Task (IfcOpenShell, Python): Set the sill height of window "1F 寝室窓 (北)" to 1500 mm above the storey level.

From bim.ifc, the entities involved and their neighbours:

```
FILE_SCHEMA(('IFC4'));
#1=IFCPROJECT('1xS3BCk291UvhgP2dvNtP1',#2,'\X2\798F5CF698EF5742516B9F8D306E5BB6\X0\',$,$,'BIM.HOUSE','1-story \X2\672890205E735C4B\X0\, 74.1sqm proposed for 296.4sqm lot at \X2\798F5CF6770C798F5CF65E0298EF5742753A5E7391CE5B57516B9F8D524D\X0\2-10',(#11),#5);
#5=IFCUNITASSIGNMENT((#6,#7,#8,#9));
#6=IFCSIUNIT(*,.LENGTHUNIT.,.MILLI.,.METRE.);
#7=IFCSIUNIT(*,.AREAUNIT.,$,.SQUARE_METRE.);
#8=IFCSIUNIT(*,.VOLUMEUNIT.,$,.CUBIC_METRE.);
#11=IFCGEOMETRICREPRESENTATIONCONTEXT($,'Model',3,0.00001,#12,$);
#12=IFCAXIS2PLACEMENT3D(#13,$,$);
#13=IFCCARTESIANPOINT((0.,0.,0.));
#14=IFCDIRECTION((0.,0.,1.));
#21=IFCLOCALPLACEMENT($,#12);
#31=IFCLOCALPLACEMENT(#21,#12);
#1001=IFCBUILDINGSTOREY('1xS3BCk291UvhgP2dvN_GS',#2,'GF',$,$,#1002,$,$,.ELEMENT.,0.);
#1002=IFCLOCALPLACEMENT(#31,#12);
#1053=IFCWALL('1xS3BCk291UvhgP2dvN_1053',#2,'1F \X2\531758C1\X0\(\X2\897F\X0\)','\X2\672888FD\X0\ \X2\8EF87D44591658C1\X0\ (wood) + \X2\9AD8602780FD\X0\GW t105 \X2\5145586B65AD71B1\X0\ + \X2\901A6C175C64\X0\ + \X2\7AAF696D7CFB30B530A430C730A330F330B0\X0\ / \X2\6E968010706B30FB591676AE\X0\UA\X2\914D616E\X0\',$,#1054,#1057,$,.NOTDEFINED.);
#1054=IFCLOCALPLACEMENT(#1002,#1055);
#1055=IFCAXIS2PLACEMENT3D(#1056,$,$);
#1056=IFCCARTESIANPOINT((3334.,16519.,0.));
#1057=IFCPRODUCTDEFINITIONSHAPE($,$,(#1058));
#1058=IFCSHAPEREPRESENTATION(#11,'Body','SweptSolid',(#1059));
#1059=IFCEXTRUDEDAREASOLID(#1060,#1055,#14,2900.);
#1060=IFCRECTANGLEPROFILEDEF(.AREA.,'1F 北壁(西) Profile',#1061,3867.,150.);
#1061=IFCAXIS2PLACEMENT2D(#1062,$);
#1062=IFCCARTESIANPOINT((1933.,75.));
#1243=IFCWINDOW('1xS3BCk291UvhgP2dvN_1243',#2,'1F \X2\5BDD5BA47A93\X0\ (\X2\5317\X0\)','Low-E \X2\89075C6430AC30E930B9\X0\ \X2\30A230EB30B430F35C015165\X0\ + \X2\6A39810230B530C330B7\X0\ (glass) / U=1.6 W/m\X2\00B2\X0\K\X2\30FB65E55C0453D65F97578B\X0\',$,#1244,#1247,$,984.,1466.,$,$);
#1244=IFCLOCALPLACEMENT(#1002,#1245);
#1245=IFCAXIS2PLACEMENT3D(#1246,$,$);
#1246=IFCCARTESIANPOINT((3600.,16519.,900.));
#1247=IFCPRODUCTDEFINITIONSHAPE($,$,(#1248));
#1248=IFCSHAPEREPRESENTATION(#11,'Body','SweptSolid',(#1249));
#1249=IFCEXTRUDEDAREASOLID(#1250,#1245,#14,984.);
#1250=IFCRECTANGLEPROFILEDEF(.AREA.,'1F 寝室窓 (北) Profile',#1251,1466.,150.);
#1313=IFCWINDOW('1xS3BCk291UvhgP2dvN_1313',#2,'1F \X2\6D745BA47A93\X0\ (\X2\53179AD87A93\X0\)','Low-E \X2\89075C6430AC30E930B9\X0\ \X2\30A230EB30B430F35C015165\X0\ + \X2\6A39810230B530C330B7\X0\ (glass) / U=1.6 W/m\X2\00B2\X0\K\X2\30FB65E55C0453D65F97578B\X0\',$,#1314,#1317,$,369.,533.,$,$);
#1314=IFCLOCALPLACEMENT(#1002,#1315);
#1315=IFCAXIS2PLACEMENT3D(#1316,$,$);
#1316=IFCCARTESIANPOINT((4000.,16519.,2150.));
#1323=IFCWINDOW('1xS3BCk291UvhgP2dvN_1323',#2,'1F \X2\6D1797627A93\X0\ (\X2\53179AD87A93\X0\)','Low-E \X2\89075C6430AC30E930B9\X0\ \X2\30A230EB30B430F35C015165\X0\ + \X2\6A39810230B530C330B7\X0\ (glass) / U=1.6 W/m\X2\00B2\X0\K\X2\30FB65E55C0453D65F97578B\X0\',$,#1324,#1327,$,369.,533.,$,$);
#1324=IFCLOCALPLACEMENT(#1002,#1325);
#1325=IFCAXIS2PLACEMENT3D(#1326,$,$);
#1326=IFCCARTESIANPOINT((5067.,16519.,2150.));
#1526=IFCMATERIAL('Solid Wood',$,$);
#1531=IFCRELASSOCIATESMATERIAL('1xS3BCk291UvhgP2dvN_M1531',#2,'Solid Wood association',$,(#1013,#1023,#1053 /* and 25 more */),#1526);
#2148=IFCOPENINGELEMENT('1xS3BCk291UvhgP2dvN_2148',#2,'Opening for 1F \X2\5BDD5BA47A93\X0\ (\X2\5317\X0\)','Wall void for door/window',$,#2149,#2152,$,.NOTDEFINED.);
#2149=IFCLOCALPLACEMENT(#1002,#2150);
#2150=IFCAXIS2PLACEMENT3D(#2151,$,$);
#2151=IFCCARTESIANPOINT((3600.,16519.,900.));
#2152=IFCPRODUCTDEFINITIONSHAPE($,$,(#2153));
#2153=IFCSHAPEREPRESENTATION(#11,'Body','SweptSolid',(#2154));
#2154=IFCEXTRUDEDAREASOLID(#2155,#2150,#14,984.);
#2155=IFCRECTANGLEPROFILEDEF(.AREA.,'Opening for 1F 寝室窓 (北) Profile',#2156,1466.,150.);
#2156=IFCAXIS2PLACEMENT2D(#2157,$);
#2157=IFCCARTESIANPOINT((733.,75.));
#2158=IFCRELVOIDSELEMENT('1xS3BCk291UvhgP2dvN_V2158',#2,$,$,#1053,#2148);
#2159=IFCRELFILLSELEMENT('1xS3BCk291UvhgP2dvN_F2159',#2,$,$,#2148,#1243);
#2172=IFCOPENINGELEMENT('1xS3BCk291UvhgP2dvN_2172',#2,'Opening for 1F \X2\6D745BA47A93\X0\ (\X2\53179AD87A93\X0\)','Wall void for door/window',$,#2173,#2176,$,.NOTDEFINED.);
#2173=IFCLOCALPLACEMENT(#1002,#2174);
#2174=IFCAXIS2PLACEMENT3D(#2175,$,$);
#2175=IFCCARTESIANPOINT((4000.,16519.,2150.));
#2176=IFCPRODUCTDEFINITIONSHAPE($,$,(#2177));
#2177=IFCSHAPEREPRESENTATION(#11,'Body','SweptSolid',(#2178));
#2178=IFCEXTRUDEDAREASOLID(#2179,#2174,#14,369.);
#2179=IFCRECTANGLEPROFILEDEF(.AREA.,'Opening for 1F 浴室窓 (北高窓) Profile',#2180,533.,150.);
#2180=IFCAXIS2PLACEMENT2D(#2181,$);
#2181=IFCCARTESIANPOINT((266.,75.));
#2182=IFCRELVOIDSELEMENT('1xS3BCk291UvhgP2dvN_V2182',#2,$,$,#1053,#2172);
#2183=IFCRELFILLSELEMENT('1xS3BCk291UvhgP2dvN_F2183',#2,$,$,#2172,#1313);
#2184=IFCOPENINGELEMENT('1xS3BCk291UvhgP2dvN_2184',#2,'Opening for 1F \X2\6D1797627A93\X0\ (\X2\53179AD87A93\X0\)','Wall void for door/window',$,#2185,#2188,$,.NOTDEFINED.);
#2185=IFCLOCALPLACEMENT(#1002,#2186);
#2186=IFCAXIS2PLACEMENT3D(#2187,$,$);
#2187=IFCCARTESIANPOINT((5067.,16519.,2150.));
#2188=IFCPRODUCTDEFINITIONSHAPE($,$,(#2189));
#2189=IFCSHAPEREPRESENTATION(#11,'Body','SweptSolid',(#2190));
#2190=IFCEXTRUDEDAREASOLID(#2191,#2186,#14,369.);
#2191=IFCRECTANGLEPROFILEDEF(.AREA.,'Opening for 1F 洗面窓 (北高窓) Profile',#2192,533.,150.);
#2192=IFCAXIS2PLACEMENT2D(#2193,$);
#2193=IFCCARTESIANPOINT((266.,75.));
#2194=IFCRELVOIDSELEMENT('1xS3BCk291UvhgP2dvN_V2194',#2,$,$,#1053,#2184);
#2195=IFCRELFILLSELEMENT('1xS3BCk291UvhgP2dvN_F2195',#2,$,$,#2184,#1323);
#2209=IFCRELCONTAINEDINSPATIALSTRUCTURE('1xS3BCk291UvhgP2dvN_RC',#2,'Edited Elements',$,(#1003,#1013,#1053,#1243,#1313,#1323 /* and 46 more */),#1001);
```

```python
import numpy as np
import ifcopenshell
import ifcopenshell.api.geometry
import ifcopenshell.geom
import ifcopenshell.util.element
import ifcopenshell.util.placement
import ifcopenshell.util.shape
import ifcopenshell.util.unit

model = ifcopenshell.open("bim.ifc")
unit_scale = ifcopenshell.util.unit.calculate_unit_scale(model)

window = model.by_guid("1xS3BCk291UvhgP2dvN_1243")
opening = window.FillsVoids[0].RelatingOpeningElement
storey = ifcopenshell.util.element.get_container(window, ifc_class="IfcBuildingStorey")
level = ifcopenshell.util.placement.get_local_placement(storey.ObjectPlacement)[2, 3]

# The opening's origin need not be at the sill, so measure its lowest point.
shape = ifcopenshell.geom.create_shape(ifcopenshell.geom.settings(), opening)
bottom = ifcopenshell.util.shape.get_shape_bottom_elevation(shape, shape.geometry) / unit_scale
dz = level + 1500.0 - bottom

shift = np.array([0.0, 0.0, dz])
# The window is not placed relative to its opening, so move both.
for product in (opening, window):
    matrix = ifcopenshell.util.placement.get_local_placement(product.ObjectPlacement)
    matrix[:3, 3] += shift
    ifcopenshell.api.geometry.edit_object_placement(model, product=product, matrix=matrix, is_si=False)

print(f"moved by {dz * unit_scale:+.3f} m")

model.write("bim_updated.ifc")
```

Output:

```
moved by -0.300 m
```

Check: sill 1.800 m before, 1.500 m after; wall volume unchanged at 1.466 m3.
